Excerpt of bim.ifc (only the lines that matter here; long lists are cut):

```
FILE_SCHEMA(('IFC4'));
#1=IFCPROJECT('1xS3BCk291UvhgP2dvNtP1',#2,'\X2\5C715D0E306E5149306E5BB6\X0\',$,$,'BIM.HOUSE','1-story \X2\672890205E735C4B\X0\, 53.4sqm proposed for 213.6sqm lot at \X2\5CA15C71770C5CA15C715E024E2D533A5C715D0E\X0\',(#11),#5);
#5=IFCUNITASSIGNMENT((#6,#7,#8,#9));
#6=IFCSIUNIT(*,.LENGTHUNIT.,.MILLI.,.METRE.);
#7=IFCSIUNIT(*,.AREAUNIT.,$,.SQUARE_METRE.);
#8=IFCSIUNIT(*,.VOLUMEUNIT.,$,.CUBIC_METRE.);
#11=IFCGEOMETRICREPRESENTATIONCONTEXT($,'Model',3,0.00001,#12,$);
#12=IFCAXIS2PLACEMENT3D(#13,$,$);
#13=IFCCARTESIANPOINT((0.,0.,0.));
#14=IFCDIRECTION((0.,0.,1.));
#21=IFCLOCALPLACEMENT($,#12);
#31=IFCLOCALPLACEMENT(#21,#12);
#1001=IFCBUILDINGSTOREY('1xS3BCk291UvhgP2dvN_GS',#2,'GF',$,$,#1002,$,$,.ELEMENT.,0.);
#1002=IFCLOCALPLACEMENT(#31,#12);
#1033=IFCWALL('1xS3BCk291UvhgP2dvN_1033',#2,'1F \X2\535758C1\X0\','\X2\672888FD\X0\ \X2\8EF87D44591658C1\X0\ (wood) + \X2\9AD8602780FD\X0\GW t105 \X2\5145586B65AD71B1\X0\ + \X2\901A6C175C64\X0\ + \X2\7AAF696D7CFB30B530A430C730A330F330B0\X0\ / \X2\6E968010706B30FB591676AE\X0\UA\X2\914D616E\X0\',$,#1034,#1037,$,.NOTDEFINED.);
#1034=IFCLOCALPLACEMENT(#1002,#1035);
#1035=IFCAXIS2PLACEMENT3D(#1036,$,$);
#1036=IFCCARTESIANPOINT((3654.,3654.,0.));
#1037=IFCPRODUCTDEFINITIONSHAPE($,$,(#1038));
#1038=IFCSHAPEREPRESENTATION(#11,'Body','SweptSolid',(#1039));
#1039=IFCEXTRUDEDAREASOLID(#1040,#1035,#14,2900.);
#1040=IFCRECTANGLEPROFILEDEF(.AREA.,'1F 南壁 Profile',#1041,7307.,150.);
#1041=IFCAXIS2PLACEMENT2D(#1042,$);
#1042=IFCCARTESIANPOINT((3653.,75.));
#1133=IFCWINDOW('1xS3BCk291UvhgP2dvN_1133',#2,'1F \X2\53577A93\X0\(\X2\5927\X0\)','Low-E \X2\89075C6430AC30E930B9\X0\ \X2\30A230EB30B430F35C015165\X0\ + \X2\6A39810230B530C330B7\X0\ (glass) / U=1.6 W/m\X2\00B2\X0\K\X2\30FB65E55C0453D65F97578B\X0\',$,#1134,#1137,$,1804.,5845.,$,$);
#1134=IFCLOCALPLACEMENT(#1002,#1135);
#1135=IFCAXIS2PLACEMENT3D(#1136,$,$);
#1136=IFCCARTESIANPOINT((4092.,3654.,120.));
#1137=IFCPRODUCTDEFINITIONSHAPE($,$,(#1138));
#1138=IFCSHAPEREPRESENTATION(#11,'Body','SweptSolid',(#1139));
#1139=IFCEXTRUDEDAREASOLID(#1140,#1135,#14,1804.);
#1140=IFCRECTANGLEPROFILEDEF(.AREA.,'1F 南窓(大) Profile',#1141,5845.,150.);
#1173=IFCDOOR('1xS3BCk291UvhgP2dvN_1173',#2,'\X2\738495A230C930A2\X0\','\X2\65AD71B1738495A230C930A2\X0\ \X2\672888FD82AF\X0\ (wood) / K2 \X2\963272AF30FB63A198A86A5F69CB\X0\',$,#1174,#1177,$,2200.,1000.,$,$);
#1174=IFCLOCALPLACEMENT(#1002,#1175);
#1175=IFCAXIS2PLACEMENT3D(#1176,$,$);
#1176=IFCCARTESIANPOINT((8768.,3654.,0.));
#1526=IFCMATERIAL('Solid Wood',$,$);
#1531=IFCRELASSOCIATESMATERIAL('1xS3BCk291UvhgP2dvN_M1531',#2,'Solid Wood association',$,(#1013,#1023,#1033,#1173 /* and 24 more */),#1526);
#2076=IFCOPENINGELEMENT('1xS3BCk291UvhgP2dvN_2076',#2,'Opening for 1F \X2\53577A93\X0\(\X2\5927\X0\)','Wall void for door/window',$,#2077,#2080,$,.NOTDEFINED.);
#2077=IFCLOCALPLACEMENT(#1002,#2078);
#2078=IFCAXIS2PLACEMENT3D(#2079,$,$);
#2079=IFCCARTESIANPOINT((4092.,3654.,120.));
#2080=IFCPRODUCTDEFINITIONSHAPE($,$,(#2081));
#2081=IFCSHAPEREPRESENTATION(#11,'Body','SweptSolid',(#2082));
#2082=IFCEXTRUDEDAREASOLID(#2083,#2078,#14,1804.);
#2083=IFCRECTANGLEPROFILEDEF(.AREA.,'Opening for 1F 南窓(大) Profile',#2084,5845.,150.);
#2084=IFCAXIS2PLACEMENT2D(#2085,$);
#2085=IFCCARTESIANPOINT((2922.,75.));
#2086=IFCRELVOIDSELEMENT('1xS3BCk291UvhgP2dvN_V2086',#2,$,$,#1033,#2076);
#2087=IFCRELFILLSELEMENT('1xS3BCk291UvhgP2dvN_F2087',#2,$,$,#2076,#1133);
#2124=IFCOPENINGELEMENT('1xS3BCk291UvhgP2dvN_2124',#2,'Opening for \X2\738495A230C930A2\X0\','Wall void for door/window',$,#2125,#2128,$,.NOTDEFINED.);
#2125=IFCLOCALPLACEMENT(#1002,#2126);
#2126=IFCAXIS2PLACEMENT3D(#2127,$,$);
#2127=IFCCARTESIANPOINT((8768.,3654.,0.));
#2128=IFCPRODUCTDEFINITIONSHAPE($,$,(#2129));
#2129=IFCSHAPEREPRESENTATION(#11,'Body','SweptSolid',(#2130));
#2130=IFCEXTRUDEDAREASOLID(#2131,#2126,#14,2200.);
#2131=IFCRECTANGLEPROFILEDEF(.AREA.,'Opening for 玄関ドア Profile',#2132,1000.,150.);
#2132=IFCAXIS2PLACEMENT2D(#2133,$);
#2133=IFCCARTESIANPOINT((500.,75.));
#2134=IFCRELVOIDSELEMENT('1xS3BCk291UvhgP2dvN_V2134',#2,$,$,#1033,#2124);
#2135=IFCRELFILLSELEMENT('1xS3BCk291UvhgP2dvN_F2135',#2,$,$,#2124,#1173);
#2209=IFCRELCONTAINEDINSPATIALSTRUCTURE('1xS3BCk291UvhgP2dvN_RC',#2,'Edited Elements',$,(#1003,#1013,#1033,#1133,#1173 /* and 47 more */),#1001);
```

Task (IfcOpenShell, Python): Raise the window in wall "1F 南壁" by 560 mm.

```python
import numpy as np
import ifcopenshell
import ifcopenshell.api.geometry
import ifcopenshell.util.placement
import ifcopenshell.util.unit

model = ifcopenshell.open("bim.ifc")
unit_scale = ifcopenshell.util.unit.calculate_unit_scale(model)

window = model.by_guid("1xS3BCk291UvhgP2dvN_1133")
opening = window.FillsVoids[0].RelatingOpeningElement
dz = 560.0

shift = np.array([0.0, 0.0, dz])
# The window is not placed relative to its opening, so move both.
for product in (opening, window):
    matrix = ifcopenshell.util.placement.get_local_placement(product.ObjectPlacement)
    matrix[:3, 3] += shift
    ifcopenshell.api.geometry.edit_object_placement(model, product=product, matrix=matrix, is_si=False)

print(f"moved by {dz * unit_scale:+.3f} m")

model.write("bim-out.ifc")
```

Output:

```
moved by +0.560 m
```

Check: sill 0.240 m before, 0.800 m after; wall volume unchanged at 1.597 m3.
